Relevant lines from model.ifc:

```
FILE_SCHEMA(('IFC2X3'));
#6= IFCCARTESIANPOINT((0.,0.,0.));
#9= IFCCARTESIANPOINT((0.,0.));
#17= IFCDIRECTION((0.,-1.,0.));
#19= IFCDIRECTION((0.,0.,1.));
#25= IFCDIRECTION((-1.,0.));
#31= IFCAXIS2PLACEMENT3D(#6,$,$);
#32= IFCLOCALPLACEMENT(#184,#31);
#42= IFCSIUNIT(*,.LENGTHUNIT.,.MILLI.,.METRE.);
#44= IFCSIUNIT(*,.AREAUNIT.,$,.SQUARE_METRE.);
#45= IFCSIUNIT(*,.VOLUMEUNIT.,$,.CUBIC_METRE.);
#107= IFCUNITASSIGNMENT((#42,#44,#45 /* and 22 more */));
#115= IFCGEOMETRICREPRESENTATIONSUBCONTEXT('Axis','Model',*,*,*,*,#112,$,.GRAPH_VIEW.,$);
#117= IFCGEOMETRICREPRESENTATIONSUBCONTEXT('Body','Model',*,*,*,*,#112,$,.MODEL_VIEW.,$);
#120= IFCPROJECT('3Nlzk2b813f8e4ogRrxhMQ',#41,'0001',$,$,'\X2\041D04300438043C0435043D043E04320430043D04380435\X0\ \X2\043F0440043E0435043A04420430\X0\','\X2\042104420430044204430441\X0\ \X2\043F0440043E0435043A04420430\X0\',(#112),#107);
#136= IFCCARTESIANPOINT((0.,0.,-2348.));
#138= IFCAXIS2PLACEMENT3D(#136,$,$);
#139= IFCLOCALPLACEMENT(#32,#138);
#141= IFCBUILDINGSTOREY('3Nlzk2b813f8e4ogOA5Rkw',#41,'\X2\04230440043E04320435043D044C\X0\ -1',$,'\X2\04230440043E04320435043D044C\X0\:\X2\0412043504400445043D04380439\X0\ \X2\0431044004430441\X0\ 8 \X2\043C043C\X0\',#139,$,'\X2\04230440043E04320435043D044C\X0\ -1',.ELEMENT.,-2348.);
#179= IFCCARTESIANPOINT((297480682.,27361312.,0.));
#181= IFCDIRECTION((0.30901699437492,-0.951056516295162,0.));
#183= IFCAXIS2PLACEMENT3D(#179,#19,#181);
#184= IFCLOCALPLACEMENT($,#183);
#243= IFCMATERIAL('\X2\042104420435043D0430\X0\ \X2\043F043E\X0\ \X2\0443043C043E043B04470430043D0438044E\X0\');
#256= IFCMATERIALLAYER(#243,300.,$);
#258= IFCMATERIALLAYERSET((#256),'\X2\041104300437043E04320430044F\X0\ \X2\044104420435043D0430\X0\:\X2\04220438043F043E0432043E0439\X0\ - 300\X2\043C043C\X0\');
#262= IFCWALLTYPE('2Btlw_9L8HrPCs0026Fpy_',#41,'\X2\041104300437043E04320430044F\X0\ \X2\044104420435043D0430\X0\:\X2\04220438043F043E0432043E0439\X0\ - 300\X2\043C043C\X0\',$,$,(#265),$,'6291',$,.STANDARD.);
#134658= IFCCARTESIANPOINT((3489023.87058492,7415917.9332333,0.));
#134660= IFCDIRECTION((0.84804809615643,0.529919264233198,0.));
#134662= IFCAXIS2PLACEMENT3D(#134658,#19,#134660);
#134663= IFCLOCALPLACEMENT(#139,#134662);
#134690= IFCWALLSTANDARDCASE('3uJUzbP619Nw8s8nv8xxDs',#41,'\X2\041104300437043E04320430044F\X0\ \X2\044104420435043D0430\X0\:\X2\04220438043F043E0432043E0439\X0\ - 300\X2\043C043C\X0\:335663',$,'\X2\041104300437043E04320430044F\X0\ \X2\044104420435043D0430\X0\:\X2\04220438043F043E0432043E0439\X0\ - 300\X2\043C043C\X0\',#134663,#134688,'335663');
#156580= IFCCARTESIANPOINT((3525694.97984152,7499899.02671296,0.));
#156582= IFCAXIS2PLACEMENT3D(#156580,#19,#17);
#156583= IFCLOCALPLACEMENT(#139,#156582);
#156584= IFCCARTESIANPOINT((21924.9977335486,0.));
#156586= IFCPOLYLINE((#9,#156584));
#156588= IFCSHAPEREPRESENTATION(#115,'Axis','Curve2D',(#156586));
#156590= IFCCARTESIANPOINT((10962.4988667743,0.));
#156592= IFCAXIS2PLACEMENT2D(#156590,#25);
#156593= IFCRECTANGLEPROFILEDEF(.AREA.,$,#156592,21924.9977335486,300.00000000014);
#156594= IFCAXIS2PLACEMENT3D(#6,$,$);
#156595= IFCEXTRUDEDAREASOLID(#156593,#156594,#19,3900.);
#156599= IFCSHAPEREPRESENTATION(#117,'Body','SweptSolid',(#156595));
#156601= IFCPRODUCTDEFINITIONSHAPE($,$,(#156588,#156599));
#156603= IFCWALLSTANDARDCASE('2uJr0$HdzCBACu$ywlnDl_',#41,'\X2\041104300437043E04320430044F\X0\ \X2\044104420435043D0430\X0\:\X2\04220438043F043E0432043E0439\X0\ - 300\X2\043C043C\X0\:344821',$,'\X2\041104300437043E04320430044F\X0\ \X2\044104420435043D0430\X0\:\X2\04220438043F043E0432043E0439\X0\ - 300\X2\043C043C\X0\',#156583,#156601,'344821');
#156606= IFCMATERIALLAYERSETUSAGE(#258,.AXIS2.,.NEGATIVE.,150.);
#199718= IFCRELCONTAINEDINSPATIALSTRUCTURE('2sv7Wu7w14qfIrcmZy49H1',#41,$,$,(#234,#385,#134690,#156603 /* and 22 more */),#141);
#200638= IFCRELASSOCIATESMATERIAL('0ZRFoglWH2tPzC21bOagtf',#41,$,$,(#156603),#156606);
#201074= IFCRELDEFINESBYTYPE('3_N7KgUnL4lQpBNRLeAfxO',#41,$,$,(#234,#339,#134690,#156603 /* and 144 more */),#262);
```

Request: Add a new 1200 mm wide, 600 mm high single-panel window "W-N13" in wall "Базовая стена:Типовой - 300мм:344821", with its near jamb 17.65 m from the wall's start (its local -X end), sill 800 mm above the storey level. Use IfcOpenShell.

```python
import numpy as np
import ifcopenshell
import ifcopenshell.api.feature
import ifcopenshell.api.geometry
import ifcopenshell.api.root
import ifcopenshell.api.spatial
import ifcopenshell.api.type
import ifcopenshell.geom
import ifcopenshell.util.element
import ifcopenshell.util.placement
import ifcopenshell.util.representation
import ifcopenshell.util.shape
import ifcopenshell.util.unit

model = ifcopenshell.open("model.ifc")
unit_scale = ifcopenshell.util.unit.calculate_unit_scale(model)
settings = ifcopenshell.geom.settings()


def volume(element):
    """Net volume in cubic metres, openings subtracted."""
    shape = ifcopenshell.geom.create_shape(settings, element)
    return ifcopenshell.util.shape.get_volume(shape.geometry)


wall = model.by_id(156603)
storey = ifcopenshell.util.element.get_container(wall, ifc_class="IfcBuildingStorey")
context = ifcopenshell.util.representation.get_context(model, "Model", "Body", "MODEL_VIEW")
before = volume(wall)

width, height, from_end, sill = 1.2, 0.6, 17.65, 0.8  # metres

# The wall runs along its own X axis, and the end named is its -X end.
wall_shape = ifcopenshell.geom.create_shape(settings, wall)
x, y, z = ifcopenshell.util.shape.get_vertices(wall_shape.geometry).T
start = x.min() + from_end
face, thickness = float(y.min()), float(y.max() - y.min())
wall_matrix = ifcopenshell.util.placement.get_local_placement(wall.ObjectPlacement)
level = ifcopenshell.util.placement.get_local_placement(storey.ObjectPlacement)[2, 3]


def in_wall(x, y):
    """Placement at x, y metres in the wall's axes, at sill height."""
    matrix = wall_matrix.copy()
    matrix[:, 3] = wall_matrix @ np.array([x / unit_scale, y / unit_scale, 0.0, 1.0])
    matrix[2, 3] = level + sill / unit_scale
    return matrix


# Opening: a box that overshoots both wall faces by 50 mm.
opening = ifcopenshell.api.root.create_entity(model, ifc_class="IfcOpeningElement")
box = ifcopenshell.api.geometry.add_wall_representation(
    model, context=context, length=width, height=height, thickness=thickness + 0.1
)
ifcopenshell.api.geometry.assign_representation(model, product=opening, representation=box)
ifcopenshell.api.geometry.edit_object_placement(model, product=opening, matrix=in_wall(start, face - 0.05), is_si=False)
ifcopenshell.api.feature.add_feature(model, feature=opening, element=wall)

window = ifcopenshell.api.root.create_entity(model, ifc_class="IfcWindow", name="W-N13")
window.OverallWidth, window.OverallHeight = width / unit_scale, height / unit_scale
body = ifcopenshell.api.geometry.add_window_representation(
    model,
    context=context,
    overall_width=window.OverallWidth,
    overall_height=window.OverallHeight,
    partition_type="SINGLE_PANEL",
)
ifcopenshell.api.geometry.assign_representation(model, product=window, representation=body)
ifcopenshell.api.spatial.assign_container(model, products=[window], relating_structure=storey)
fills = ifcopenshell.api.feature.add_filling(model, opening=opening, element=window)
fills.OwnerHistory = window.OwnerHistory  # required in IFC2X3

# IFC2X3 keeps the operation on the window style.
style = ifcopenshell.api.root.create_entity(model, ifc_class="IfcWindowStyle", name="W-N13")
style.OperationType, style.ConstructionType = "SINGLE_PANEL", "NOTDEFINED"
style.ParameterTakesPrecedence = style.Sizeable = False
ifcopenshell.api.type.assign_type(model, related_objects=[window], relating_type=style)

# Centre the window in the wall's thickness.
ifcopenshell.api.geometry.edit_object_placement(model, product=window, matrix=in_wall(start, face), is_si=False)
window_shape = ifcopenshell.geom.create_shape(settings, window)
depth = ifcopenshell.util.shape.get_vertices(window_shape.geometry)[:, 1]
offset = face + thickness / 2 - (depth.min() + depth.max()) / 2
ifcopenshell.api.geometry.edit_object_placement(model, product=window, matrix=in_wall(start, offset), is_si=False)

after = volume(wall)

print(f"wall volume {before:.3f} -> {after:.3f} m3")

model.write("model_edited.ifc")
```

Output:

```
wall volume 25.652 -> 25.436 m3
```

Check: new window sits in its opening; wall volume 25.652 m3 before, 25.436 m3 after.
